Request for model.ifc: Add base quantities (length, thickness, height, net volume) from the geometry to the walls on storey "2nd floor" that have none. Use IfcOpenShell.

First a look at what the model holds.

```python
import ifcopenshell
import ifcopenshell.util.element
import ifcopenshell.util.unit

model = ifcopenshell.open("model.ifc")
print(model.schema)
for unit_type in ("LENGTHUNIT", "AREAUNIT", "VOLUMEUNIT"):
    print(unit_type, ifcopenshell.util.unit.calculate_unit_scale(model, unit_type))
storey = next(s for s in model.by_type("IfcBuildingStorey") if s.Name == "2nd floor")
walls = [e for e in ifcopenshell.util.element.get_decomposition(storey) if e.is_a("IfcWall")]
for e in sorted(walls, key=lambda e: e.id()):
    print(e.id(), e.is_a(), e.Name, list(ifcopenshell.util.element.get_psets(e, qtos_only=True)), sep=" | ")
```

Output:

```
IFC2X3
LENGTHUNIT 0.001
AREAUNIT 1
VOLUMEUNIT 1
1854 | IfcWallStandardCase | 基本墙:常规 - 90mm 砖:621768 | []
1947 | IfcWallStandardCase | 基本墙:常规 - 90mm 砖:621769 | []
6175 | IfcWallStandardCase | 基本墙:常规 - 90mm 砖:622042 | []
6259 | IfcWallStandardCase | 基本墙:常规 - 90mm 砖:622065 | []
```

```python
import ifcopenshell
import ifcopenshell.api.pset
import ifcopenshell.geom
import ifcopenshell.util.element
import ifcopenshell.util.shape
import ifcopenshell.util.unit

model = ifcopenshell.open("model.ifc")
unit_scale = ifcopenshell.util.unit.calculate_unit_scale(model)
volume_scale = ifcopenshell.util.unit.calculate_unit_scale(model, "VOLUMEUNIT")
settings = ifcopenshell.geom.settings()

storey = next(s for s in model.by_type("IfcBuildingStorey") if s.Name == "2nd floor")
walls = [e for e in ifcopenshell.util.element.get_decomposition(storey) if e.is_a("IfcWall")]

for e in sorted(walls, key=lambda e: e.id()):
    if ifcopenshell.util.element.get_psets(e, qtos_only=True, should_inherit=False):
        continue
    # Geometry comes back in metres, in the element's own axes.
    shape = ifcopenshell.geom.create_shape(settings, e)
    values = {
        "Length": ifcopenshell.util.shape.get_x(shape.geometry) / unit_scale,
        "Width": ifcopenshell.util.shape.get_y(shape.geometry) / unit_scale,
        "Height": ifcopenshell.util.shape.get_z(shape.geometry) / unit_scale,
        "NetVolume": ifcopenshell.util.shape.get_volume(shape.geometry) / volume_scale,
    }
    qto = ifcopenshell.api.pset.add_qto(model, product=e, name="BaseQuantities")
    ifcopenshell.api.pset.edit_qto(model, qto=qto, properties=values)
    print(e.id(), {k: round(v, 3) for k, v in values.items()})

model.write("model_rev.ifc")
```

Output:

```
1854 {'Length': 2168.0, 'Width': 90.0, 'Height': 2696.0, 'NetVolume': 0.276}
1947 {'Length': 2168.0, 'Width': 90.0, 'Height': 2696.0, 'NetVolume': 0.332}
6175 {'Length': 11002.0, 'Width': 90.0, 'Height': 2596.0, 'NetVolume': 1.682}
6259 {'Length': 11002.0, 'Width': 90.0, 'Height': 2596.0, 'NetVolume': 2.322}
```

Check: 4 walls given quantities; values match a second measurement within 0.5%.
